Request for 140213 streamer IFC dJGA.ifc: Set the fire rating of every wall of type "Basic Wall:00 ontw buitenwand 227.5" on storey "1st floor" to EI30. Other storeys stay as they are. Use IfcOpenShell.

First a look at what the model holds.

```python
import ifcopenshell
import ifcopenshell.util.element

model = ifcopenshell.open("140213 streamer IFC dJGA.ifc")
print(model.schema)
storey = next(s for s in model.by_type("IfcBuildingStorey") if s.Name == "1st floor")
walls = [e for e in ifcopenshell.util.element.get_decomposition(storey) if e.is_a("IfcWall")]
seen = {}
for e in walls:
    element_type = ifcopenshell.util.element.get_type(e)
    key = (element_type.Name if element_type != e and element_type else None, ifcopenshell.util.element.get_pset(e, "Pset_WallCommon", "FireRating"))
    seen[key] = seen.get(key, 0) + 1
for (name, value), count in sorted(seen.items(), key=str):
    print(count, "x", name, "|", value)
```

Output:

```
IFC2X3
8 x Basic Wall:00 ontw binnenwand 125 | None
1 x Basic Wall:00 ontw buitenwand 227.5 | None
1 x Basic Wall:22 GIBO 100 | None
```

```python
import ifcopenshell
import ifcopenshell.api.pset
import ifcopenshell.util.element

model = ifcopenshell.open("140213 streamer IFC dJGA.ifc")

storey = next(s for s in model.by_type("IfcBuildingStorey") if s.Name == "1st floor")
walls = [e for e in ifcopenshell.util.element.get_decomposition(storey) if e.is_a("IfcWall")]

count = 0
for e in walls:
    element_type = ifcopenshell.util.element.get_type(e)
    if element_type in (None, e) or element_type.Name != "Basic Wall:00 ontw buitenwand 227.5":
        continue
    # add_pset returns the element's existing set when there is one.
    pset = ifcopenshell.api.pset.add_pset(model, product=e, name="Pset_WallCommon")
    ifcopenshell.api.pset.edit_pset(model, pset=pset, properties={"FireRating": "EI30"})
    count += 1

print(count, "walls updated")

model.write("140213 streamer IFC dJGA_edited.ifc")
```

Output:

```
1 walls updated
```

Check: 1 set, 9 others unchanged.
